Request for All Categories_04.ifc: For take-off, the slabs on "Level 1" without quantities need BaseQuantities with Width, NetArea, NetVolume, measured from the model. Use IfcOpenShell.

First a look at what the model holds.

```python
import ifcopenshell
import ifcopenshell.util.element
import ifcopenshell.util.unit

model = ifcopenshell.open("All Categories_04.ifc")
print(model.schema)
for unit_type in ("LENGTHUNIT", "AREAUNIT", "VOLUMEUNIT"):
    print(unit_type, ifcopenshell.util.unit.calculate_unit_scale(model, unit_type))
storey = next(s for s in model.by_type("IfcBuildingStorey") if s.Name == "Level 1")
slabs = [e for e in ifcopenshell.util.element.get_decomposition(storey) if e.is_a("IfcSlab")]
for e in sorted(slabs, key=lambda e: e.id()):
    print(e.id(), e.is_a(), e.Name, list(ifcopenshell.util.element.get_psets(e, qtos_only=True)), sep=" | ")
```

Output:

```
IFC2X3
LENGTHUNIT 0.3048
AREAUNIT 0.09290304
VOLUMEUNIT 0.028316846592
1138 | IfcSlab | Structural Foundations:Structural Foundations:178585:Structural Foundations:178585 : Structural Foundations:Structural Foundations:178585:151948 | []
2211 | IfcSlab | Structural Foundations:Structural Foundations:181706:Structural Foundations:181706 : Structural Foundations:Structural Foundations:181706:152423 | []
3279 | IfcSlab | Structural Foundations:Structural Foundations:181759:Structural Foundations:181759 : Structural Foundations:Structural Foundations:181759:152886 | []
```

```python
import ifcopenshell
import ifcopenshell.api.pset
import ifcopenshell.geom
import ifcopenshell.util.element
import ifcopenshell.util.shape
import ifcopenshell.util.unit

model = ifcopenshell.open("All Categories_04.ifc")
unit_scale = ifcopenshell.util.unit.calculate_unit_scale(model)
area_scale = ifcopenshell.util.unit.calculate_unit_scale(model, "AREAUNIT")
volume_scale = ifcopenshell.util.unit.calculate_unit_scale(model, "VOLUMEUNIT")
settings = ifcopenshell.geom.settings()

storey = next(s for s in model.by_type("IfcBuildingStorey") if s.Name == "Level 1")
slabs = [e for e in ifcopenshell.util.element.get_decomposition(storey) if e.is_a("IfcSlab")]

for e in sorted(slabs, key=lambda e: e.id()):
    if ifcopenshell.util.element.get_psets(e, qtos_only=True, should_inherit=False):
        continue
    # Geometry comes back in metres, in the element's own axes.
    shape = ifcopenshell.geom.create_shape(settings, e)
    values = {
        "Width": ifcopenshell.util.shape.get_z(shape.geometry) / unit_scale,
        "NetArea": ifcopenshell.util.shape.get_footprint_area(shape.geometry) / area_scale,
        "NetVolume": ifcopenshell.util.shape.get_volume(shape.geometry) / volume_scale,
    }
    qto = ifcopenshell.api.pset.add_qto(model, product=e, name="BaseQuantities")
    ifcopenshell.api.pset.edit_qto(model, qto=qto, properties=values)
    print(e.id(), {k: round(v, 3) for k, v in values.items()})

model.write("All Categories_04_v2.ifc")
```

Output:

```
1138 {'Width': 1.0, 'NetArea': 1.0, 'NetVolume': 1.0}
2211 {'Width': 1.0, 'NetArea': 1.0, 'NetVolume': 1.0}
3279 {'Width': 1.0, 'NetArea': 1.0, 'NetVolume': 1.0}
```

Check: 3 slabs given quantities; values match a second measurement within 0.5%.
